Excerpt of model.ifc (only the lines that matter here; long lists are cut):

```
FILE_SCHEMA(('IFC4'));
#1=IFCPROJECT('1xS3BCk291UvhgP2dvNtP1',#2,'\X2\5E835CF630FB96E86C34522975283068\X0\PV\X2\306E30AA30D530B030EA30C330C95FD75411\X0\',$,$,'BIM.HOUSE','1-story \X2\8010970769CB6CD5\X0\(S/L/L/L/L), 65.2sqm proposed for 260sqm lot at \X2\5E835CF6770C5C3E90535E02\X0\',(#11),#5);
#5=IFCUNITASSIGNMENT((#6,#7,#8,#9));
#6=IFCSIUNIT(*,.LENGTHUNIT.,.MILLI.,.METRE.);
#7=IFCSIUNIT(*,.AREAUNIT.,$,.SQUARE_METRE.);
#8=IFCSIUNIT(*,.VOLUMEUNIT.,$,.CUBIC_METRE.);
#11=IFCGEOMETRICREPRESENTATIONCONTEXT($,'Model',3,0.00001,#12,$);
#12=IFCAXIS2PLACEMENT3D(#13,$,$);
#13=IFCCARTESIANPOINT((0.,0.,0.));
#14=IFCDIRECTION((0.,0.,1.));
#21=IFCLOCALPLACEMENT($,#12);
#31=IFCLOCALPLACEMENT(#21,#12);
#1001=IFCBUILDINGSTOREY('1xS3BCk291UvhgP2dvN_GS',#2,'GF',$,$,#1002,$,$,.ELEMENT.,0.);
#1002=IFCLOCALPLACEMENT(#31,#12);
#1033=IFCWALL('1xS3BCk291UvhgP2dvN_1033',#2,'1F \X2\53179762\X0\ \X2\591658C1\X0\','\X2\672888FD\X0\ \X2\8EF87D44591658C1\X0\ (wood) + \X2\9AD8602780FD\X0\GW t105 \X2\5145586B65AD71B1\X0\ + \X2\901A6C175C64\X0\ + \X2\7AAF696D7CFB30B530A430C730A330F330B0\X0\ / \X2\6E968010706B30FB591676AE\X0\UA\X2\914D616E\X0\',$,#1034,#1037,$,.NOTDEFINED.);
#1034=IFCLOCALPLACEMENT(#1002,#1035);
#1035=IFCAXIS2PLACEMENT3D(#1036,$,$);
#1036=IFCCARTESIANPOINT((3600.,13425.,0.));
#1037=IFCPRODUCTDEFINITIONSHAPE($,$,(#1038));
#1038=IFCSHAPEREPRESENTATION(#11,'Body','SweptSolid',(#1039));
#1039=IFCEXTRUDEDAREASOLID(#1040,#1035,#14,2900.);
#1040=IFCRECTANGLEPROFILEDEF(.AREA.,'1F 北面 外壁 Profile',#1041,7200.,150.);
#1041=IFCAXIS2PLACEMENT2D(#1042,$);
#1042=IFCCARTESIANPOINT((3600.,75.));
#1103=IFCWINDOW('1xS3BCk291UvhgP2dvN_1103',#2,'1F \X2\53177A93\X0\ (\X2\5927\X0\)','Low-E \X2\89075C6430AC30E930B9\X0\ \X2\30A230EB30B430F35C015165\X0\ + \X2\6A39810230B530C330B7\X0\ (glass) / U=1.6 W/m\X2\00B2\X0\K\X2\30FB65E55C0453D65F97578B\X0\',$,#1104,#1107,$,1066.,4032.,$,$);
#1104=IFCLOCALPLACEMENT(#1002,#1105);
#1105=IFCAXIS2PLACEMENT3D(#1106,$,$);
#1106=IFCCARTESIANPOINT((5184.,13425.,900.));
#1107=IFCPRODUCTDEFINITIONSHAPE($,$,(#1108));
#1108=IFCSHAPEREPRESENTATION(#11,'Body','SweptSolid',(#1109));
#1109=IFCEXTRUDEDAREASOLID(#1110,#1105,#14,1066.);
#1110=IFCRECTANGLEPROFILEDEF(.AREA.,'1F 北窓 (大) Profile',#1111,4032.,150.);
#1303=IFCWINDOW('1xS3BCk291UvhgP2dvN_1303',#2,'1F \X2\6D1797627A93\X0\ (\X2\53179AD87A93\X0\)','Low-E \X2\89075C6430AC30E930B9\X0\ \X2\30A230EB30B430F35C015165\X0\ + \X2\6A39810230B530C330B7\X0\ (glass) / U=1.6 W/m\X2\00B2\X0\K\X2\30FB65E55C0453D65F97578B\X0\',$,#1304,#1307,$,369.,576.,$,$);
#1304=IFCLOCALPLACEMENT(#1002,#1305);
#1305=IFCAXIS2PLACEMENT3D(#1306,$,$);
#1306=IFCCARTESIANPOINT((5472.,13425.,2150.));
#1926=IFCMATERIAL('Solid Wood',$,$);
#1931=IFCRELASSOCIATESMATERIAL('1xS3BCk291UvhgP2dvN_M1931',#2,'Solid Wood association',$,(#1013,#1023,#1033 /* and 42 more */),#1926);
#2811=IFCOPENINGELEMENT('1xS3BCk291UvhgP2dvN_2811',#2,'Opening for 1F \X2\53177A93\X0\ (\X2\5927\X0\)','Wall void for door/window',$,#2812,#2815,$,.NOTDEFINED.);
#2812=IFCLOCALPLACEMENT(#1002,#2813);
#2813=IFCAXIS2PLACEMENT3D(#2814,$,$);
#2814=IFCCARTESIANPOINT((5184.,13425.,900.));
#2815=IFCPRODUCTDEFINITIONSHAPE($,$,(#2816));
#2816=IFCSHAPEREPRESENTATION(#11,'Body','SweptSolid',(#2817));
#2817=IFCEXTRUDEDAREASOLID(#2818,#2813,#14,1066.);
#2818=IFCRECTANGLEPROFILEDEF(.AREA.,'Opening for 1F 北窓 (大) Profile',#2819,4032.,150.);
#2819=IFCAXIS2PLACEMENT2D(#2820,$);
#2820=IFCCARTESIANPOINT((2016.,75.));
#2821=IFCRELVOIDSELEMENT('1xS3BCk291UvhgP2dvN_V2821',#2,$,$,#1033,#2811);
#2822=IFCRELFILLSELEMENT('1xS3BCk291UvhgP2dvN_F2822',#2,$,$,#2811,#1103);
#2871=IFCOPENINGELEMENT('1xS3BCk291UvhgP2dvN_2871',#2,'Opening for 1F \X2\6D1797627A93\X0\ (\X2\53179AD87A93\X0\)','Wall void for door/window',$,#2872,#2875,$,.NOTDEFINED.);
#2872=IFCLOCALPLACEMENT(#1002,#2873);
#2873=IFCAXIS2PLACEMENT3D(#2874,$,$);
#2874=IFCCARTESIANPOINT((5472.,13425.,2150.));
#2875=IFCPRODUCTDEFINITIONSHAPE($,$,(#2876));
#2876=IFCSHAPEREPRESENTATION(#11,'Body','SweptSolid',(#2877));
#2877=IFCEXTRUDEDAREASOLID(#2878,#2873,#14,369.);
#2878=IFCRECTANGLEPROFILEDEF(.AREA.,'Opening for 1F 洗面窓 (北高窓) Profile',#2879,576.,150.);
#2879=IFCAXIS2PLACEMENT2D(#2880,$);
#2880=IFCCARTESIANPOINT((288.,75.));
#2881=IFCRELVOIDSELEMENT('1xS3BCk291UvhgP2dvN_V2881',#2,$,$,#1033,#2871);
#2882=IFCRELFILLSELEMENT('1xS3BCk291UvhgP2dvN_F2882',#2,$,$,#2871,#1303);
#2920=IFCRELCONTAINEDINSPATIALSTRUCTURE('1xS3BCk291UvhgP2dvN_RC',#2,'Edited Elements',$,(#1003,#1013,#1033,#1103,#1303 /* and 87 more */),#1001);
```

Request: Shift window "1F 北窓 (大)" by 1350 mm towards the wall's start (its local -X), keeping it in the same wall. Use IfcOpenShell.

```python
import ifcopenshell
import ifcopenshell.api.geometry
import ifcopenshell.util.placement

model = ifcopenshell.open("model.ifc")

window = model.by_guid("1xS3BCk291UvhgP2dvN_1103")
opening = window.FillsVoids[0].RelatingOpeningElement
wall = opening.VoidsElements[0].RelatingBuildingElement

wall_matrix = ifcopenshell.util.placement.get_local_placement(wall.ObjectPlacement)
shift = wall_matrix[:3, 0] * -1350.0
before = ifcopenshell.util.placement.get_local_placement(window.ObjectPlacement)[:3, 3].copy()

# The window is not placed relative to its opening, so move both.
for product in (opening, window):
    matrix = ifcopenshell.util.placement.get_local_placement(product.ObjectPlacement)
    matrix[:3, 3] += shift
    ifcopenshell.api.geometry.edit_object_placement(model, product=product, matrix=matrix, is_si=False)

after = ifcopenshell.util.placement.get_local_placement(window.ObjectPlacement)[:3, 3]
print("window moved by", (after - before).round(3) + 0.0)

model.write("model_updated.ifc")
```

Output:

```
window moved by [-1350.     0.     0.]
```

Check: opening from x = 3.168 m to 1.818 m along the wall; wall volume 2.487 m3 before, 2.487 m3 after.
